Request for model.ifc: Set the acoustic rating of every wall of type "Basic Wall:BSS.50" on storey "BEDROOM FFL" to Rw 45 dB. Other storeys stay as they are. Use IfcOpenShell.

First a look at what the model holds.

```python
import ifcopenshell
import ifcopenshell.util.element

model = ifcopenshell.open("model.ifc")
print(model.schema)
storey = next(s for s in model.by_type("IfcBuildingStorey") if s.Name == "BEDROOM FFL")
walls = [e for e in ifcopenshell.util.element.get_decomposition(storey) if e.is_a("IfcWall")]
seen = {}
for e in walls:
    element_type = ifcopenshell.util.element.get_type(e)
    key = (element_type.Name if element_type != e and element_type else None, ifcopenshell.util.element.get_pset(e, "Pset_WallCommon", "AcousticRating"))
    seen[key] = seen.get(key, 0) + 1
for (name, value), count in sorted(seen.items(), key=str):
    print(count, "x", name, "|", value)
```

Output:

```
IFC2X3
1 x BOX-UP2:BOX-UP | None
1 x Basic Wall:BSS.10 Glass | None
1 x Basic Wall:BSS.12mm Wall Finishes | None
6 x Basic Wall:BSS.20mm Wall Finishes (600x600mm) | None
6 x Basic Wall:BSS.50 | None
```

```python
import ifcopenshell
import ifcopenshell.api.pset
import ifcopenshell.util.element

model = ifcopenshell.open("model.ifc")

storey = next(s for s in model.by_type("IfcBuildingStorey") if s.Name == "BEDROOM FFL")
walls = [e for e in ifcopenshell.util.element.get_decomposition(storey) if e.is_a("IfcWall")]

count = 0
for e in walls:
    element_type = ifcopenshell.util.element.get_type(e)
    if element_type in (None, e) or element_type.Name != "Basic Wall:BSS.50":
        continue
    # add_pset returns the element's existing set when there is one.
    pset = ifcopenshell.api.pset.add_pset(model, product=e, name="Pset_WallCommon")
    ifcopenshell.api.pset.edit_pset(model, pset=pset, properties={"AcousticRating": "Rw 45 dB"})
    count += 1

print(count, "walls updated")

model.write("model_updated.ifc")
```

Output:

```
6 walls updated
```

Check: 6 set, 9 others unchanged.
